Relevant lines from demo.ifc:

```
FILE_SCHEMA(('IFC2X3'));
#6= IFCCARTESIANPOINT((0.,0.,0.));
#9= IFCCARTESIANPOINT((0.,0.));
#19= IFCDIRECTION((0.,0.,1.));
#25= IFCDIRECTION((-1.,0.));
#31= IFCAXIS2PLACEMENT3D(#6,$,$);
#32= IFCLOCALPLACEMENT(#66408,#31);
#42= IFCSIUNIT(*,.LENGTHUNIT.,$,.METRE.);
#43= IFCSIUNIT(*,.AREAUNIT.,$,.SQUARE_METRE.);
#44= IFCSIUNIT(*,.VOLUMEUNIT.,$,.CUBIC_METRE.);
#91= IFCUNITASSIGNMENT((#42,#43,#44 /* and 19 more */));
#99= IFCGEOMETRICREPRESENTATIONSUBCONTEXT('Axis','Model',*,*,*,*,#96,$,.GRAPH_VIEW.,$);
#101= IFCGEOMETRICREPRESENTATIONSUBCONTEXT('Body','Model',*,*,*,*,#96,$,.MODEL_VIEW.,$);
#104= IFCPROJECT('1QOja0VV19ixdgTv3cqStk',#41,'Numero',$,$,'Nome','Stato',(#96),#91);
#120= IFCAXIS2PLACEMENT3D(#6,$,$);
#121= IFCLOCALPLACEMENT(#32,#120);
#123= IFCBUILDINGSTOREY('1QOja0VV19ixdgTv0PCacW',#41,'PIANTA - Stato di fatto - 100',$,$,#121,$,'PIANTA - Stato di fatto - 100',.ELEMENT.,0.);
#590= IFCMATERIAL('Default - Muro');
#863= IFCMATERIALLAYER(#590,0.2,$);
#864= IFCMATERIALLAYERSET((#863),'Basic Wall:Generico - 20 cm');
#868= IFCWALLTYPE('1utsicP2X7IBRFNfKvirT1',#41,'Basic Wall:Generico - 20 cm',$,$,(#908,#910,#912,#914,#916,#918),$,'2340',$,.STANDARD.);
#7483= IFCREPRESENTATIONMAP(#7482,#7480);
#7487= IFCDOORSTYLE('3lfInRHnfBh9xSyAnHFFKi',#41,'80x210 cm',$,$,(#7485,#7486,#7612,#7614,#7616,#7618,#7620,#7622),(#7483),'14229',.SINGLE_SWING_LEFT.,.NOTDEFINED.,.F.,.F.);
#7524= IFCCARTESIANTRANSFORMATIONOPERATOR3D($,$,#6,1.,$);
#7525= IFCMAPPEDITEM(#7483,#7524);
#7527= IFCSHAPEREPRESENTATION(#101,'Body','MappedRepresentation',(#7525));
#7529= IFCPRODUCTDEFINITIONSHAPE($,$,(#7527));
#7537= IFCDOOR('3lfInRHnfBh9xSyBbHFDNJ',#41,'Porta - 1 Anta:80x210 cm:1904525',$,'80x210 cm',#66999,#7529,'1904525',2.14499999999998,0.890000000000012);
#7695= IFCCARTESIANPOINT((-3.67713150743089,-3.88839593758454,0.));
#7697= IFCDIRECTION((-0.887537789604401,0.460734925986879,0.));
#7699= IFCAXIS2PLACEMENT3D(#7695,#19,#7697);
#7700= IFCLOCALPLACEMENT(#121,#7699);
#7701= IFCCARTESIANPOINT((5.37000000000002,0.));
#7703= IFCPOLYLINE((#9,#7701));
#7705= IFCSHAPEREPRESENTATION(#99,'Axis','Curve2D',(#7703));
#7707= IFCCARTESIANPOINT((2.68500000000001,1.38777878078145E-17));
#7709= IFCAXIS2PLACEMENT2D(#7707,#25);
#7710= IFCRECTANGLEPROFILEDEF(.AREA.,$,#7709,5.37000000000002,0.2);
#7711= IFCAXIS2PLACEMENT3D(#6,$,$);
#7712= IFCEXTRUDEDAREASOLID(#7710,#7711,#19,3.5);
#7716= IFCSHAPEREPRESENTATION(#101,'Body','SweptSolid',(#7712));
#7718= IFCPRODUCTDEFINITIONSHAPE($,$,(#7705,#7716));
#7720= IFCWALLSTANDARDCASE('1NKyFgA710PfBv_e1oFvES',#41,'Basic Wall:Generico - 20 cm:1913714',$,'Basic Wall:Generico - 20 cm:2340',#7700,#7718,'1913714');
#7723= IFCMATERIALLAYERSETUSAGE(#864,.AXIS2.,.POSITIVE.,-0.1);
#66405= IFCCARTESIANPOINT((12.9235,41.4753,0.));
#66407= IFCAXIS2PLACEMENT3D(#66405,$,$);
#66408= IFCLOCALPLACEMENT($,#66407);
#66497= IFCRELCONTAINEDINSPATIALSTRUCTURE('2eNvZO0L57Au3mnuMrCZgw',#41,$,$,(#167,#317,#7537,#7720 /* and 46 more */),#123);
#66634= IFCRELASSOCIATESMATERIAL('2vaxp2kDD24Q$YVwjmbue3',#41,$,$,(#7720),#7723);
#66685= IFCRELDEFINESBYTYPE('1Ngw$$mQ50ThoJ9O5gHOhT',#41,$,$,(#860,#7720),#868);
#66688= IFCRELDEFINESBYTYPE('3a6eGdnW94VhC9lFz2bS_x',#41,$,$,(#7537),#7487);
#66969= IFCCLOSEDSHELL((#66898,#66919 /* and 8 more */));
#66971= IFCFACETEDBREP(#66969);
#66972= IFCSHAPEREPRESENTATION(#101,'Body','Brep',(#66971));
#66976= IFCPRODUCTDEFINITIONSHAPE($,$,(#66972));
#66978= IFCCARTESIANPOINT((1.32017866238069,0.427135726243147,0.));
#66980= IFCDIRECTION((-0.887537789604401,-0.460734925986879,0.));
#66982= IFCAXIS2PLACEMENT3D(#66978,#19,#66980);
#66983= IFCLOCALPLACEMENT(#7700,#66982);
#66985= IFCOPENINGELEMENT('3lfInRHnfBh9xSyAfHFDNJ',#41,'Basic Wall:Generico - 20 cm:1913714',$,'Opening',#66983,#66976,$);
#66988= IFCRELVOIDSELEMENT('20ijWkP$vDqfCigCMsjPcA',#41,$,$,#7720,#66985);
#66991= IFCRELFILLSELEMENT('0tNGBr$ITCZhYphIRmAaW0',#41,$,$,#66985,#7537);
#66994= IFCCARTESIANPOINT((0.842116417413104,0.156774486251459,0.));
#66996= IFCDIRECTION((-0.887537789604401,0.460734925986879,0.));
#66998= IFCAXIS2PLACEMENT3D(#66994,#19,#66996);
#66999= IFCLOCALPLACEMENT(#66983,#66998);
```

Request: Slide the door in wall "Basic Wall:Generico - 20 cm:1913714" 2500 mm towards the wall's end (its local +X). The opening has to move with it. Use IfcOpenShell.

```python
import ifcopenshell
import ifcopenshell.api.geometry
import ifcopenshell.util.placement
import ifcopenshell.util.unit

model = ifcopenshell.open("demo.ifc")
unit_scale = ifcopenshell.util.unit.calculate_unit_scale(model)

door = model.by_guid("3lfInRHnfBh9xSyBbHFDNJ")
opening = door.FillsVoids[0].RelatingOpeningElement
wall = opening.VoidsElements[0].RelatingBuildingElement

wall_matrix = ifcopenshell.util.placement.get_local_placement(wall.ObjectPlacement)
shift = wall_matrix[:3, 0] * 2.5 / unit_scale
before = ifcopenshell.util.placement.get_local_placement(door.ObjectPlacement)[:3, 3].copy()

# The door is placed relative to its opening, so it follows when the opening moves.
matrix = ifcopenshell.util.placement.get_local_placement(opening.ObjectPlacement)
matrix[:3, 3] += shift
ifcopenshell.api.geometry.edit_object_placement(
    model, product=opening, matrix=matrix, is_si=False, should_transform_children=True
)

after = ifcopenshell.util.placement.get_local_placement(door.ObjectPlacement)[:3, 3]
print("door moved by", (after - before).round(3) + 0.0)

model.write("demo_v2.ifc")
```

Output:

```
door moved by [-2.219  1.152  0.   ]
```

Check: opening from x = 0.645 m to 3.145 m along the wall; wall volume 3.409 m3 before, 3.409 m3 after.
